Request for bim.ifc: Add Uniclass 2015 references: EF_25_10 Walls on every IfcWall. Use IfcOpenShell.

First a look at what the model holds.

```python
import ifcopenshell

model = ifcopenshell.open("bim.ifc")
print(model.schema)
print("classifications:", [c.Name for c in model.by_type("IfcClassification")])
for ifc_class in ("IfcDoor", "IfcRoof", "IfcStair", "IfcWall", "IfcWindow"):
    print(ifc_class, len(model.by_type(ifc_class)))
```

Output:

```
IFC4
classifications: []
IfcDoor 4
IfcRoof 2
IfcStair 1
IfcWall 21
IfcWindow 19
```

```python
import ifcopenshell
import ifcopenshell.api.classification

model = ifcopenshell.open("bim.ifc")

system = ifcopenshell.api.classification.add_classification(model, classification="Uniclass 2015")

codes = {
    "IfcWall": ("EF_25_10", "Walls"),
}
for ifc_class, (code, name) in codes.items():
    products = model.by_type(ifc_class)
    ifcopenshell.api.classification.add_reference(
        model, products=products, classification=system, identification=code, name=name
    )
    print(code, len(products))

model.write("bim_v2.ifc")
```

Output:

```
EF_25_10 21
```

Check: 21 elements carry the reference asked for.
